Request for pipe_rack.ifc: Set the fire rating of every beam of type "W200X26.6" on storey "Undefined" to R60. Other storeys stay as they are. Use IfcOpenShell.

First a look at what the model holds.

```python
import ifcopenshell
import ifcopenshell.util.element

model = ifcopenshell.open("pipe_rack.ifc")
print(model.schema)
storey = next(s for s in model.by_type("IfcBuildingStorey") if s.Name == "Undefined")
beams = [e for e in ifcopenshell.util.element.get_decomposition(storey) if e.is_a("IfcBeam")]
seen = {}
for e in beams:
    element_type = ifcopenshell.util.element.get_type(e)
    key = (element_type.Name if element_type != e and element_type else None, ifcopenshell.util.element.get_pset(e, "Pset_BeamCommon", "FireRating"))
    seen[key] = seen.get(key, 0) + 1
for (name, value), count in sorted(seen.items(), key=str):
    print(count, "x", name, "|", value)
```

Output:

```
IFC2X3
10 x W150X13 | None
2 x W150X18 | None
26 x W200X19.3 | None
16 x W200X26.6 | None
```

```python
import ifcopenshell
import ifcopenshell.api.pset
import ifcopenshell.util.element

model = ifcopenshell.open("pipe_rack.ifc")

storey = next(s for s in model.by_type("IfcBuildingStorey") if s.Name == "Undefined")
beams = [e for e in ifcopenshell.util.element.get_decomposition(storey) if e.is_a("IfcBeam")]

count = 0
for e in beams:
    element_type = ifcopenshell.util.element.get_type(e)
    if element_type in (None, e) or element_type.Name != "W200X26.6":
        continue
    found = ifcopenshell.util.element.get_pset(e, "Pset_BeamCommon", should_inherit=False)
    if found:
        pset = model.by_id(found["id"])
        if len(ifcopenshell.util.element.get_elements_by_pset(pset)) > 1:
            pset = ifcopenshell.api.pset.unshare_pset(model, products=[e], pset=pset)[0]
    else:
        pset = ifcopenshell.api.pset.add_pset(model, product=e, name="Pset_BeamCommon")
    ifcopenshell.api.pset.edit_pset(model, pset=pset, properties={"FireRating": "R60"})
    count += 1

print(count, "beams updated")

model.write("pipe_rack-out.ifc")
```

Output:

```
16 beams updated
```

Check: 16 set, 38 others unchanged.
